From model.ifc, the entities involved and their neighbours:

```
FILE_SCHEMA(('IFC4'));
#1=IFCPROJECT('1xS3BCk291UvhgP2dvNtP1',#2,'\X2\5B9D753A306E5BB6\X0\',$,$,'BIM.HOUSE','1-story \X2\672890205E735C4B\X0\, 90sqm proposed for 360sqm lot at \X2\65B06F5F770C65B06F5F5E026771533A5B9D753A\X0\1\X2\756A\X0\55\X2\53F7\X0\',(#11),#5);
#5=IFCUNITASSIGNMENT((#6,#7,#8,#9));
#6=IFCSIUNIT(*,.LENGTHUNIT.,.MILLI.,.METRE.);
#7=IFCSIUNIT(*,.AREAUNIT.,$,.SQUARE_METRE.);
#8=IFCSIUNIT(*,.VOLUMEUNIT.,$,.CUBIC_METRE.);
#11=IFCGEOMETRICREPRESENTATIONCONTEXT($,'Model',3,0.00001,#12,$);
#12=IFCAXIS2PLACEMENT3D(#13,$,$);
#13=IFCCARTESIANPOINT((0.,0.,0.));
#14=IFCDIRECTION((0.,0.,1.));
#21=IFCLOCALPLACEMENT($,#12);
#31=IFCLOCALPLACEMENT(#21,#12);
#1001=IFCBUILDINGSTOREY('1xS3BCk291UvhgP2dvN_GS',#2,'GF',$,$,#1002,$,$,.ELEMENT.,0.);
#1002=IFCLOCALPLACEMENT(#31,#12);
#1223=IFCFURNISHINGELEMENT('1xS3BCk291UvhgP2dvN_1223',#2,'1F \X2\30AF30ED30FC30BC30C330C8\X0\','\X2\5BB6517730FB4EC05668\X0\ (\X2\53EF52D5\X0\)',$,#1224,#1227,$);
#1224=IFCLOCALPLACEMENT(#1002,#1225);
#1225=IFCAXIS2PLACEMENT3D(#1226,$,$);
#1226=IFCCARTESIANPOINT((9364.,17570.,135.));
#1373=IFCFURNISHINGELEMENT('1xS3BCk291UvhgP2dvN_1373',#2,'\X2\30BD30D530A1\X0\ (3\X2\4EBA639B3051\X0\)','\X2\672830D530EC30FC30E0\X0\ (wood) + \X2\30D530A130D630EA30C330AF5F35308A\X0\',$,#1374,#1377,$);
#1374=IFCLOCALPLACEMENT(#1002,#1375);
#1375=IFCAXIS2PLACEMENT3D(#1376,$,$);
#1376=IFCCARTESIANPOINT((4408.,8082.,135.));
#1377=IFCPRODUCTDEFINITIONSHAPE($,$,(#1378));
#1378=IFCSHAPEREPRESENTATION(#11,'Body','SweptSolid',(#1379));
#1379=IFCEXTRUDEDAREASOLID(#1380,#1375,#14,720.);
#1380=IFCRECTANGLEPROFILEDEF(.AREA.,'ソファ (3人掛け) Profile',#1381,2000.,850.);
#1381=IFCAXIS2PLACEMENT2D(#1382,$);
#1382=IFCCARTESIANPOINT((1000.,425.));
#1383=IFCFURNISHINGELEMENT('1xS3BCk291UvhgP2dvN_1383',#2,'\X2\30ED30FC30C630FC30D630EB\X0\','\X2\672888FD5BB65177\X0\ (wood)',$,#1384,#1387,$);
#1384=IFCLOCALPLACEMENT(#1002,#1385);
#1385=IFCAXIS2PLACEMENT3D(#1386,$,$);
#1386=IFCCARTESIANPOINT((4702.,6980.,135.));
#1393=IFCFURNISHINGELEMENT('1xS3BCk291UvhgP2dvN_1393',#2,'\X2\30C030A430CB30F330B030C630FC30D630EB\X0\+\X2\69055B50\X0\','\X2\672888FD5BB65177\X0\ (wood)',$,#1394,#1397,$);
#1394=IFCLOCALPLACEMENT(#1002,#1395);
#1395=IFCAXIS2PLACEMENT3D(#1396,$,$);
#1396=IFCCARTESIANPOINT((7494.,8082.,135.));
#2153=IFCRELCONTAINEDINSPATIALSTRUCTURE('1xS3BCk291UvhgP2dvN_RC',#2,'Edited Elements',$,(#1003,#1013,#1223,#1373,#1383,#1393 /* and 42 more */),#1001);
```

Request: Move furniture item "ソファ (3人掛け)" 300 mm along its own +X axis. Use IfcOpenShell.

```python
import ifcopenshell
import ifcopenshell.api.geometry
import ifcopenshell.util.placement

model = ifcopenshell.open("model.ifc")

item = model.by_id(1373)
matrix = ifcopenshell.util.placement.get_local_placement(item.ObjectPlacement)
matrix[:3, 3] += matrix[:3, 0] * 300.0
ifcopenshell.api.geometry.edit_object_placement(model, product=item, matrix=matrix, is_si=False)

print(ifcopenshell.util.placement.get_local_placement(item.ObjectPlacement).round(3) + 0.0)

model.write("model_v2.ifc")
```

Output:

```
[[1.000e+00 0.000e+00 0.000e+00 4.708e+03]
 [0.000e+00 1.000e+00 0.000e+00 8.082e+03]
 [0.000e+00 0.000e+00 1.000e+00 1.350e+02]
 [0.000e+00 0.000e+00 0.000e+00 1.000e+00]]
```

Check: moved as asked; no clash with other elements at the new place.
